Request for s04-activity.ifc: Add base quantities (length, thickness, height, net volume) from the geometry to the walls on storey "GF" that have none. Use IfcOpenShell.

First a look at what the model holds.

```python
import ifcopenshell
import ifcopenshell.util.element
import ifcopenshell.util.unit

model = ifcopenshell.open("s04-activity.ifc")
print(model.schema)
for unit_type in ("LENGTHUNIT", "AREAUNIT", "VOLUMEUNIT"):
    print(unit_type, ifcopenshell.util.unit.calculate_unit_scale(model, unit_type))
storey = next(s for s in model.by_type("IfcBuildingStorey") if s.Name == "GF")
walls = [e for e in ifcopenshell.util.element.get_decomposition(storey) if e.is_a("IfcWall")]
for e in sorted(walls, key=lambda e: e.id()):
    print(e.id(), e.is_a(), e.Name, list(ifcopenshell.util.element.get_psets(e, qtos_only=True)), sep=" | ")
```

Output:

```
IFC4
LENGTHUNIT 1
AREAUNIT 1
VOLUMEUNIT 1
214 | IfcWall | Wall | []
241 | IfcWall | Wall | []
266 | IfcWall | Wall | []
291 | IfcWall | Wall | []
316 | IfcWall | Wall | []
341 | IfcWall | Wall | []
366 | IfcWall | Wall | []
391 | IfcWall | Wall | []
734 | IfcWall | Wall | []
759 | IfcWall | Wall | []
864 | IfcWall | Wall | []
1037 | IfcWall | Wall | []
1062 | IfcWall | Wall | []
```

```python
import ifcopenshell
import ifcopenshell.api.pset
import ifcopenshell.geom
import ifcopenshell.util.element
import ifcopenshell.util.shape
import ifcopenshell.util.unit

model = ifcopenshell.open("s04-activity.ifc")
unit_scale = ifcopenshell.util.unit.calculate_unit_scale(model)
volume_scale = ifcopenshell.util.unit.calculate_unit_scale(model, "VOLUMEUNIT")
settings = ifcopenshell.geom.settings()

storey = next(s for s in model.by_type("IfcBuildingStorey") if s.Name == "GF")
walls = [e for e in ifcopenshell.util.element.get_decomposition(storey) if e.is_a("IfcWall")]

for e in sorted(walls, key=lambda e: e.id()):
    if ifcopenshell.util.element.get_psets(e, qtos_only=True, should_inherit=False):
        continue
    # Geometry comes back in metres, in the element's own axes.
    shape = ifcopenshell.geom.create_shape(settings, e)
    values = {
        "Length": ifcopenshell.util.shape.get_x(shape.geometry) / unit_scale,
        "Width": ifcopenshell.util.shape.get_y(shape.geometry) / unit_scale,
        "Height": ifcopenshell.util.shape.get_z(shape.geometry) / unit_scale,
        "NetVolume": ifcopenshell.util.shape.get_volume(shape.geometry) / volume_scale,
    }
    qto = ifcopenshell.api.pset.add_qto(model, product=e, name="Qto_WallBaseQuantities")
    ifcopenshell.api.pset.edit_qto(model, qto=qto, properties=values)
    print(e.id(), {k: round(v, 3) for k, v in values.items()})

model.write("s04-activity_updated.ifc")
```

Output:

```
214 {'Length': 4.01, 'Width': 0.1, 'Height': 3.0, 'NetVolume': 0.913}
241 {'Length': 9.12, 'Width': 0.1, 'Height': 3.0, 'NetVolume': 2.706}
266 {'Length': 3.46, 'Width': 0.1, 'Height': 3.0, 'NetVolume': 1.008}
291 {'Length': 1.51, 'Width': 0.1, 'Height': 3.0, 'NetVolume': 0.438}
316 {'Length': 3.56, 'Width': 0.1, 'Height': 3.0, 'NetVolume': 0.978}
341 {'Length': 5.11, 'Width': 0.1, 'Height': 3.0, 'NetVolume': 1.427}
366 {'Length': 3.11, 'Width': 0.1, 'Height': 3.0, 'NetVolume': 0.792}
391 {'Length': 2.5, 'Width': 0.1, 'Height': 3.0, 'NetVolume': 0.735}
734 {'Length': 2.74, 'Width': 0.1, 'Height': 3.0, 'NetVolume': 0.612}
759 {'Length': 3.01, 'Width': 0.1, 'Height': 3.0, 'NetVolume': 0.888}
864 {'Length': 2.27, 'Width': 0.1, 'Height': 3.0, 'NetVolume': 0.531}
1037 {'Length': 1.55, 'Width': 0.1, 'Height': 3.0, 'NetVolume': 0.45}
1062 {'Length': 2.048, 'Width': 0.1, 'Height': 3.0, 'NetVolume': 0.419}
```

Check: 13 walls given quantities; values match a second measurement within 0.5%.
